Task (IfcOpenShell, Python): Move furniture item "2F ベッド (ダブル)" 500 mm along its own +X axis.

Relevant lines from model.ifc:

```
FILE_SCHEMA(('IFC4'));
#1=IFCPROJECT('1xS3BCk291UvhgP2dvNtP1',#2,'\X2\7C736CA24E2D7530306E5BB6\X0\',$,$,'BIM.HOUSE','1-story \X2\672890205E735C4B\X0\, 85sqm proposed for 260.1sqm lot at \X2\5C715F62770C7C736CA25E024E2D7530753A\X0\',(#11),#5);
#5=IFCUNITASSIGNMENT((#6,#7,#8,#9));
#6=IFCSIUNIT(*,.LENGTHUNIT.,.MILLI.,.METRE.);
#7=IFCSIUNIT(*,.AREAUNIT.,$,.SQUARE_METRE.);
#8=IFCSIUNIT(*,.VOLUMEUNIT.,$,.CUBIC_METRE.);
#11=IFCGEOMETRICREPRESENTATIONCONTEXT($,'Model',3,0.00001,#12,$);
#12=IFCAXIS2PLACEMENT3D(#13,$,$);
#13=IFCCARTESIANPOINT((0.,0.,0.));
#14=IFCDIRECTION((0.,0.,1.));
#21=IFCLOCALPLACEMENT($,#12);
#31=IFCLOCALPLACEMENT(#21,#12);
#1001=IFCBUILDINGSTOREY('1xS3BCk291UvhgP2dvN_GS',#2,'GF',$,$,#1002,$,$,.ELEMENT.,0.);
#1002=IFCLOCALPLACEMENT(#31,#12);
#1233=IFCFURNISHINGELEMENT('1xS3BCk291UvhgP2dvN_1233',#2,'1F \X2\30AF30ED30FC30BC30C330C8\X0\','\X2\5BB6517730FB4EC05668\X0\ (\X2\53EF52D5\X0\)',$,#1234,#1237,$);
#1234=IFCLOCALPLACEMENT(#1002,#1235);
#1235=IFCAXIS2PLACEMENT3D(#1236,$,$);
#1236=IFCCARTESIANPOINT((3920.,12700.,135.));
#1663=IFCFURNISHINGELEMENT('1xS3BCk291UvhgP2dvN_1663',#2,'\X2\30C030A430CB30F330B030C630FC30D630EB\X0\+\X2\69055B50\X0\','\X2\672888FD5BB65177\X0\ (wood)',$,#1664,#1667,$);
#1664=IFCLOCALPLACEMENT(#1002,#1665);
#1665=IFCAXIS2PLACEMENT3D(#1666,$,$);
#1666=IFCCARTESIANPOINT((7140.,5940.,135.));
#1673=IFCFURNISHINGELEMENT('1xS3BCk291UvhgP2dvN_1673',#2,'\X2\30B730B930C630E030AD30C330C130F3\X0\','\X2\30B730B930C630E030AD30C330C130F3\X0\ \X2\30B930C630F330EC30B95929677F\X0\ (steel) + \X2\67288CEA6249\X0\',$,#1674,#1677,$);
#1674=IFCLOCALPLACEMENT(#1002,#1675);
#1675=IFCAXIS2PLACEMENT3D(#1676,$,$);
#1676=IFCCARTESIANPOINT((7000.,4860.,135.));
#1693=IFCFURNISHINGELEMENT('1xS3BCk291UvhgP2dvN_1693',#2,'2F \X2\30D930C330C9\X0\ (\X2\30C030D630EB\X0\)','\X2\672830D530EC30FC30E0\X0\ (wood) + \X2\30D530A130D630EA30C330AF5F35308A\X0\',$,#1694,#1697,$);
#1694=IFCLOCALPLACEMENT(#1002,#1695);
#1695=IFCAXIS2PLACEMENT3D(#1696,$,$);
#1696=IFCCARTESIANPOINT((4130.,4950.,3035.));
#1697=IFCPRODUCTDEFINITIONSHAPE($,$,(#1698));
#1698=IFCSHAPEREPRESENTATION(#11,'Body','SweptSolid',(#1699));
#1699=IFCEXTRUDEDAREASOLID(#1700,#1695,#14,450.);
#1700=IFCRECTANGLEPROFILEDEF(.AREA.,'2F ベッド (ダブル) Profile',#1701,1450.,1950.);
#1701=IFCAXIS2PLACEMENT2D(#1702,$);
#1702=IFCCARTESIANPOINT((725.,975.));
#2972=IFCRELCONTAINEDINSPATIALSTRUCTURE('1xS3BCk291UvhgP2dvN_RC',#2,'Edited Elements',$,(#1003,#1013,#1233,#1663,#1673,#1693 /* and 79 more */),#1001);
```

```python
import ifcopenshell
import ifcopenshell.api.geometry
import ifcopenshell.util.placement
import ifcopenshell.util.unit

model = ifcopenshell.open("model.ifc")
unit_scale = ifcopenshell.util.unit.calculate_unit_scale(model)

item = model.by_guid("1xS3BCk291UvhgP2dvN_1693")
matrix = ifcopenshell.util.placement.get_local_placement(item.ObjectPlacement)
matrix[:3, 3] += matrix[:3, 0] * 0.5 / unit_scale
ifcopenshell.api.geometry.edit_object_placement(model, product=item, matrix=matrix, is_si=False)

print(ifcopenshell.util.placement.get_local_placement(item.ObjectPlacement).round(3) + 0.0)

model.write("model_v2.ifc")
```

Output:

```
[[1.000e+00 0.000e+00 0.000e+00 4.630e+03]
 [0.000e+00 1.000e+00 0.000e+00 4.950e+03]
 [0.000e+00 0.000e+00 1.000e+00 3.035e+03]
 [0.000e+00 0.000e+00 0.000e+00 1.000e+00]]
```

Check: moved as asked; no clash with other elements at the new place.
